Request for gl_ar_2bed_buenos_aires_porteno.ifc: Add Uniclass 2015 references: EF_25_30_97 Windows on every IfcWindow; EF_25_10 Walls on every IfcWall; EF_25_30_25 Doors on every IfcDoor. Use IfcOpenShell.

First a look at what the model holds.

```python
import ifcopenshell

model = ifcopenshell.open("gl_ar_2bed_buenos_aires_porteno.ifc")
print(model.schema)
print("classifications:", [c.Name for c in model.by_type("IfcClassification")])
for ifc_class in ("IfcDoor", "IfcRoof", "IfcStair", "IfcWall", "IfcWindow"):
    print(ifc_class, len(model.by_type(ifc_class)))
```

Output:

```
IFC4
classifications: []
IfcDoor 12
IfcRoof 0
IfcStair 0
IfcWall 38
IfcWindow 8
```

```python
import ifcopenshell
import ifcopenshell.api.classification

model = ifcopenshell.open("gl_ar_2bed_buenos_aires_porteno.ifc")

system = ifcopenshell.api.classification.add_classification(model, classification="Uniclass 2015")

codes = {
    "IfcWindow": ("EF_25_30_97", "Windows"),
    "IfcWall": ("EF_25_10", "Walls"),
    "IfcDoor": ("EF_25_30_25", "Doors"),
}
for ifc_class, (code, name) in codes.items():
    products = model.by_type(ifc_class)
    ifcopenshell.api.classification.add_reference(
        model, products=products, classification=system, identification=code, name=name
    )
    print(code, len(products))

model.write("gl_ar_2bed_buenos_aires_porteno_edited.ifc")
```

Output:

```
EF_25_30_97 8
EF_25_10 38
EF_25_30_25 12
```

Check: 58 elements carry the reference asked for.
